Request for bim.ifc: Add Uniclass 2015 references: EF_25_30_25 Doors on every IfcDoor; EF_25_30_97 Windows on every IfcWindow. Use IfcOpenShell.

First a look at what the model holds.

```python
import ifcopenshell

model = ifcopenshell.open("bim.ifc")
print(model.schema)
print("classifications:", [c.Name for c in model.by_type("IfcClassification")])
for ifc_class in ("IfcDoor", "IfcRoof", "IfcStair", "IfcWall", "IfcWindow"):
    print(ifc_class, len(model.by_type(ifc_class)))
```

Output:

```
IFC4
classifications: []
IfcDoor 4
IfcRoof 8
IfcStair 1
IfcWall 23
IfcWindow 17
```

```python
import ifcopenshell
import ifcopenshell.api.classification

model = ifcopenshell.open("bim.ifc")

system = ifcopenshell.api.classification.add_classification(model, classification="Uniclass 2015")

codes = {
    "IfcDoor": ("EF_25_30_25", "Doors"),
    "IfcWindow": ("EF_25_30_97", "Windows"),
}
for ifc_class, (code, name) in codes.items():
    products = model.by_type(ifc_class)
    ifcopenshell.api.classification.add_reference(
        model, products=products, classification=system, identification=code, name=name
    )
    print(code, len(products))

model.write("bim_updated.ifc")
```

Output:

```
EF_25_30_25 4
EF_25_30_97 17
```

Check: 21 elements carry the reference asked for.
